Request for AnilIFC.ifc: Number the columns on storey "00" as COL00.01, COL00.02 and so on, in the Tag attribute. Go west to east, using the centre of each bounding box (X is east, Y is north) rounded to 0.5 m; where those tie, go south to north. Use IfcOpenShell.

First a look at what the model holds.

```python
import ifcopenshell
import ifcopenshell.util.element
import ifcopenshell.util.placement

model = ifcopenshell.open("AnilIFC.ifc")
print(model.schema)
storey = next(s for s in model.by_type("IfcBuildingStorey") if s.Name == "00")
columns = [e for e in ifcopenshell.util.element.get_decomposition(storey) if e.is_a("IfcColumn")]
for e in sorted(columns, key=lambda e: e.id()):
    origin = ifcopenshell.util.placement.get_local_placement(e.ObjectPlacement)[:3, 3]
    print(e.id(), e.Tag, e.Name, origin.round(2) + 0.0, sep=" | ")
```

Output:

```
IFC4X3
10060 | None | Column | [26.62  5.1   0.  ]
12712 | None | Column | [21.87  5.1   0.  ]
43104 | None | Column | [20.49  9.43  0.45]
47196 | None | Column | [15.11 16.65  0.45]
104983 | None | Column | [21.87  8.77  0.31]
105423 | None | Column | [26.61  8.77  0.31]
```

```python
import ifcopenshell
import ifcopenshell.geom
import ifcopenshell.util.element
import ifcopenshell.util.shape

model = ifcopenshell.open("AnilIFC.ifc")
settings = ifcopenshell.geom.settings()
settings.set("use-world-coords", True)


def centre(element):
    shape = ifcopenshell.geom.create_shape(settings, element)
    return ifcopenshell.util.shape.get_bbox_centroid(shape.geometry)


storey = next(s for s in model.by_type("IfcBuildingStorey") if s.Name == "00")
columns = [e for e in ifcopenshell.util.element.get_decomposition(storey) if e.is_a("IfcColumn")]

# Insertion points can sit at a corner or the storey origin, so sort by the geometry (in metres).
centres = {e: centre(e) for e in columns}
columns.sort(key=lambda e: (round(centres[e][0] / 0.5), centres[e][1]))

for i, e in enumerate(columns, start=1):
    number = f"COL00.{i:02d}"
    e.Tag = number
    print(e.id(), number)

model.write("AnilIFC-out.ifc")
```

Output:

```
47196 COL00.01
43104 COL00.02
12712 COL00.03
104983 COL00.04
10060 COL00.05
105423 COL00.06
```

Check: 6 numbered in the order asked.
